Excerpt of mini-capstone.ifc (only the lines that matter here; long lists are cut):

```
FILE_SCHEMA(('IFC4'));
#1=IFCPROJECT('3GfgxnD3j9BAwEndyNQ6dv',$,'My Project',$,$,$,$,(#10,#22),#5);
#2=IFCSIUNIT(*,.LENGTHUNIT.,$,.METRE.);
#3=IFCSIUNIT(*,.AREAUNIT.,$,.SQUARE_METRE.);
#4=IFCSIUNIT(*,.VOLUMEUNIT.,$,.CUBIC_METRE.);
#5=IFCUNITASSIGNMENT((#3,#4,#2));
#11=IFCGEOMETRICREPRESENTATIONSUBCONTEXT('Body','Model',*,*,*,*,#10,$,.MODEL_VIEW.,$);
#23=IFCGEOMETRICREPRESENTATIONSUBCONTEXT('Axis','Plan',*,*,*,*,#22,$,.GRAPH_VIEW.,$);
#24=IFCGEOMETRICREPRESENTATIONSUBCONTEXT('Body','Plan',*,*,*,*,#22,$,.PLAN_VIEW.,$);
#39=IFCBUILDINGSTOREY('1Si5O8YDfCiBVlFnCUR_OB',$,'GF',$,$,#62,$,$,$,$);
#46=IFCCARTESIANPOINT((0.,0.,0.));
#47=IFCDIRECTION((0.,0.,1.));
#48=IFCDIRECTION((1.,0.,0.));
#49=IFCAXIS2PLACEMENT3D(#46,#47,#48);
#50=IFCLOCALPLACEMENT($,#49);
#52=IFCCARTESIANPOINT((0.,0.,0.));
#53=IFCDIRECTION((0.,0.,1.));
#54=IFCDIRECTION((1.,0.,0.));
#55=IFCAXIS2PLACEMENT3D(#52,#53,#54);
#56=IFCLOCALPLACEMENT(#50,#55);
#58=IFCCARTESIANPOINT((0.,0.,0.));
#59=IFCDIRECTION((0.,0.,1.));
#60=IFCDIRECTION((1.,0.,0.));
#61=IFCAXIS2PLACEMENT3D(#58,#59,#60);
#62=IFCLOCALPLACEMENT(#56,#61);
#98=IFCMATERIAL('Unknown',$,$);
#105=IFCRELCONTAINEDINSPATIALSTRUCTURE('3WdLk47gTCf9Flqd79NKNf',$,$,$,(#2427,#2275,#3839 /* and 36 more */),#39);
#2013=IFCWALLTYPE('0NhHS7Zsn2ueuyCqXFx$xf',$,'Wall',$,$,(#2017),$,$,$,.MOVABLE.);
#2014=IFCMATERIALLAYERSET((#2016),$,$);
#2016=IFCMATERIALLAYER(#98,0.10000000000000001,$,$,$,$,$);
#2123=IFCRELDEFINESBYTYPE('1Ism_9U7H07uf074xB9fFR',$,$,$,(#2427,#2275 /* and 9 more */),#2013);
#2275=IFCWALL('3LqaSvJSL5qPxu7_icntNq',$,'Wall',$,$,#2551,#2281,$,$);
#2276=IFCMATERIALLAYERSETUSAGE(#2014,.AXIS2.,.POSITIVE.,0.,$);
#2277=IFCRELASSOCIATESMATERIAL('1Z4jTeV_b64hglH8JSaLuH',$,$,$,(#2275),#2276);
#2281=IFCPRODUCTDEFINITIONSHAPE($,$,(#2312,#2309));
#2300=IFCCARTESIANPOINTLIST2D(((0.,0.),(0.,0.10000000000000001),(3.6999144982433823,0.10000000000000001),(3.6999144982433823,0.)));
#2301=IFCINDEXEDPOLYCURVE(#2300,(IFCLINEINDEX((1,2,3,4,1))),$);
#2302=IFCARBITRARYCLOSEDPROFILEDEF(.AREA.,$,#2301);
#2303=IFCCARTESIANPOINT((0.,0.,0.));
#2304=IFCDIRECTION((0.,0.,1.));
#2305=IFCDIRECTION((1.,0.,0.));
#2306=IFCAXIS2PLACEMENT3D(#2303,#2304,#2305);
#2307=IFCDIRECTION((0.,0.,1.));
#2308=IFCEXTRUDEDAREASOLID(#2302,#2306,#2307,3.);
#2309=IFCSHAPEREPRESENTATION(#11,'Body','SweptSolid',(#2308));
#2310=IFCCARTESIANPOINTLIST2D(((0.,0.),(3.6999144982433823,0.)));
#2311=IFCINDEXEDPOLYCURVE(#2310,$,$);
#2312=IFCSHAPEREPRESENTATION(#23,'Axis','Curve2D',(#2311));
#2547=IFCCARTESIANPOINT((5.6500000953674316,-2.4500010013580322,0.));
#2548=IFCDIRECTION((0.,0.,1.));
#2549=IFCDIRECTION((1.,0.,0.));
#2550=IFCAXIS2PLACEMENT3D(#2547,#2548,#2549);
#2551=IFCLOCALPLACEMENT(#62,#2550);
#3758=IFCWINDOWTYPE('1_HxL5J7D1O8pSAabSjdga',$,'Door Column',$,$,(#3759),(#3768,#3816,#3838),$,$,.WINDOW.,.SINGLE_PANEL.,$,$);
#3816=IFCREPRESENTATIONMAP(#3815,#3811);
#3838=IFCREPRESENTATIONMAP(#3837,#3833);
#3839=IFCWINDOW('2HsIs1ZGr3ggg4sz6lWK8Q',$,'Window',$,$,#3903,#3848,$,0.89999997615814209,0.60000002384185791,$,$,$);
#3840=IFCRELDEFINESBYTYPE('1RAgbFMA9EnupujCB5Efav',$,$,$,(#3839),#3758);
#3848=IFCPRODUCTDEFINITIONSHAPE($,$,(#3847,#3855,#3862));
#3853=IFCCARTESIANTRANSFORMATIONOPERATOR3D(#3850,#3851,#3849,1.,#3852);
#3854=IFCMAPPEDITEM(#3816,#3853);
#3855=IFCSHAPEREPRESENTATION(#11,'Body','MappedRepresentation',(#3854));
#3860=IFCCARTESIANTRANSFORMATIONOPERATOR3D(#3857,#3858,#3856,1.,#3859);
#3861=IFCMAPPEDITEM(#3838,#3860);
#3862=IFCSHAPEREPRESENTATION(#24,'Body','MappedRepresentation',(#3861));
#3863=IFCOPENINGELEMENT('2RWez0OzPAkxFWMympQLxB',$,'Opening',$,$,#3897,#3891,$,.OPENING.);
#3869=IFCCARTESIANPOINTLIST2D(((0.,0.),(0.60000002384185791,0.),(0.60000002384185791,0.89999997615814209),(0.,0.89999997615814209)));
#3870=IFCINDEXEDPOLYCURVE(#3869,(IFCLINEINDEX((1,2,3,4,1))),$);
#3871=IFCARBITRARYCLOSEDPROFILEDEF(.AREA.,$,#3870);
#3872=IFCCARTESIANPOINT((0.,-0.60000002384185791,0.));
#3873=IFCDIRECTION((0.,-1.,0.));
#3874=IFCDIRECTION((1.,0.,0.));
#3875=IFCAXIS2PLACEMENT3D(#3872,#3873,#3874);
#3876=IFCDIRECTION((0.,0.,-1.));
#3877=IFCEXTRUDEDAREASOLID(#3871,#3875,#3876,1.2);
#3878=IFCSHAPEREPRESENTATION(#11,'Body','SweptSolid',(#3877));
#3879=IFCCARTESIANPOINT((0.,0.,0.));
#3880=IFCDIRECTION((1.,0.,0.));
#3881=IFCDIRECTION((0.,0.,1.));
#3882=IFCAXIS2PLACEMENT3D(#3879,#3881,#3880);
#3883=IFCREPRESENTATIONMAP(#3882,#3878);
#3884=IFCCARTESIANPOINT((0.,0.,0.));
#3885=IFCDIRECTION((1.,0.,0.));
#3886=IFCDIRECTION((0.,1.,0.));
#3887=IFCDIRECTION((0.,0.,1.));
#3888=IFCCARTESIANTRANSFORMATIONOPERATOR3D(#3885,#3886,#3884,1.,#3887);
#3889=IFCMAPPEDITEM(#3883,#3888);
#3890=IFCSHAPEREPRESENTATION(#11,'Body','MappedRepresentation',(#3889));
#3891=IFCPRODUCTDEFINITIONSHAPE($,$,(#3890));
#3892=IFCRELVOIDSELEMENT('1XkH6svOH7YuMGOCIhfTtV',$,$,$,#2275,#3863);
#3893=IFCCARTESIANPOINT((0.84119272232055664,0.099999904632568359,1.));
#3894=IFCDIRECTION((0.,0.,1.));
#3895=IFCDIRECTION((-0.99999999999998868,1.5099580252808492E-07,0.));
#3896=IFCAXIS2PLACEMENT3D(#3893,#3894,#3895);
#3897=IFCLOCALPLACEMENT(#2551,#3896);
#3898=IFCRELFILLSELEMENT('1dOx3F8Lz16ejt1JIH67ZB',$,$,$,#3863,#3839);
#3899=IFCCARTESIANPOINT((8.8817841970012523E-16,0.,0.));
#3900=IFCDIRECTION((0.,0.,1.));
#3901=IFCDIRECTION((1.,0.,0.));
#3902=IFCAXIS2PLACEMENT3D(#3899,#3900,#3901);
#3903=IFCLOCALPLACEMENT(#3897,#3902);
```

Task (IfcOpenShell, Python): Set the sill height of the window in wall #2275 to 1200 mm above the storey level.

```python
import numpy as np
import ifcopenshell
import ifcopenshell.api.geometry
import ifcopenshell.geom
import ifcopenshell.util.element
import ifcopenshell.util.placement
import ifcopenshell.util.shape
import ifcopenshell.util.unit

model = ifcopenshell.open("mini-capstone.ifc")
unit_scale = ifcopenshell.util.unit.calculate_unit_scale(model)

window = model.by_guid("2HsIs1ZGr3ggg4sz6lWK8Q")
opening = window.FillsVoids[0].RelatingOpeningElement
storey = ifcopenshell.util.element.get_container(window, ifc_class="IfcBuildingStorey")
level = ifcopenshell.util.placement.get_local_placement(storey.ObjectPlacement)[2, 3]

# The opening's origin need not be at the sill, so measure its lowest point.
shape = ifcopenshell.geom.create_shape(ifcopenshell.geom.settings(), opening)
bottom = ifcopenshell.util.shape.get_shape_bottom_elevation(shape, shape.geometry) / unit_scale
dz = level + 1.2 - bottom

shift = np.array([0.0, 0.0, dz])
# The window is placed relative to its opening, so it follows when the opening moves.
matrix = ifcopenshell.util.placement.get_local_placement(opening.ObjectPlacement)
matrix[:3, 3] += shift
ifcopenshell.api.geometry.edit_object_placement(
    model, product=opening, matrix=matrix, is_si=False, should_transform_children=True
)

print(f"moved by {dz * unit_scale:+.3f} m")

model.write("mini-capstone_rev.ifc")
```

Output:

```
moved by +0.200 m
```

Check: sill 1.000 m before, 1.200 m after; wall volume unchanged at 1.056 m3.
